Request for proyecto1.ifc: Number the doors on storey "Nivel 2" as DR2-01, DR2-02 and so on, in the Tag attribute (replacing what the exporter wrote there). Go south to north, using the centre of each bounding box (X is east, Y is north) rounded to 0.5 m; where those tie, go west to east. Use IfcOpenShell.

First a look at what the model holds.

```python
import ifcopenshell
import ifcopenshell.util.element
import ifcopenshell.util.placement

model = ifcopenshell.open("proyecto1.ifc")
print(model.schema)
storey = next(s for s in model.by_type("IfcBuildingStorey") if s.Name == "Nivel 2")
doors = [e for e in ifcopenshell.util.element.get_decomposition(storey) if e.is_a("IfcDoor")]
for e in sorted(doors, key=lambda e: e.id()):
    origin = ifcopenshell.util.placement.get_local_placement(e.ObjectPlacement)[:3, 3]
    print(e.id(), e.Tag, e.Name, origin.round(2) + 0.0, sep=" | ")
```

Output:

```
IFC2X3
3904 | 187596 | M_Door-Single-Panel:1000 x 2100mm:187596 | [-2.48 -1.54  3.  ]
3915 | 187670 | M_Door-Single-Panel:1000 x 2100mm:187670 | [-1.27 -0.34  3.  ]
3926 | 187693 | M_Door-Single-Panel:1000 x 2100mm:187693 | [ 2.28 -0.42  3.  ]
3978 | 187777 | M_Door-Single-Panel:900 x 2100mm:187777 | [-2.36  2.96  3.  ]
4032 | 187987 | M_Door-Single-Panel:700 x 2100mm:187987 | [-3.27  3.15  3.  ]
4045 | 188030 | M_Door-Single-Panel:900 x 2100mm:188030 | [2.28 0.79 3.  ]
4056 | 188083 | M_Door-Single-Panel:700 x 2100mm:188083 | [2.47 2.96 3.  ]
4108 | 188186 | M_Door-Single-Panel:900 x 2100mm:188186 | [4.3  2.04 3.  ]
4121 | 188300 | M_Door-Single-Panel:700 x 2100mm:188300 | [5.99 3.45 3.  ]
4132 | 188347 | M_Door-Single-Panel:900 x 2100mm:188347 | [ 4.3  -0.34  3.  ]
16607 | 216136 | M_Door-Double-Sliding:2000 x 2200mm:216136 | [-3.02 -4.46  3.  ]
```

```python
import ifcopenshell
import ifcopenshell.geom
import ifcopenshell.util.element
import ifcopenshell.util.shape

model = ifcopenshell.open("proyecto1.ifc")
settings = ifcopenshell.geom.settings()
settings.set("use-world-coords", True)


def centre(element):
    shape = ifcopenshell.geom.create_shape(settings, element)
    return ifcopenshell.util.shape.get_bbox_centroid(shape.geometry)


storey = next(s for s in model.by_type("IfcBuildingStorey") if s.Name == "Nivel 2")
doors = [e for e in ifcopenshell.util.element.get_decomposition(storey) if e.is_a("IfcDoor")]

# Insertion points can sit at a corner or the storey origin, so sort by the geometry (in metres).
centres = {e: centre(e) for e in doors}
doors.sort(key=lambda e: (round(centres[e][1] / 0.5), centres[e][0]))

for i, e in enumerate(doors, start=1):
    number = f"DR2-{i:02d}"
    e.Tag = number
    print(e.id(), number)

model.write("proyecto1_rev.ifc")
```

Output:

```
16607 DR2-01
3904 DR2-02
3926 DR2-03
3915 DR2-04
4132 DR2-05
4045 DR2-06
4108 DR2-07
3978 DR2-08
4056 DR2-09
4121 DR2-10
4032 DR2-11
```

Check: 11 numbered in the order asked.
